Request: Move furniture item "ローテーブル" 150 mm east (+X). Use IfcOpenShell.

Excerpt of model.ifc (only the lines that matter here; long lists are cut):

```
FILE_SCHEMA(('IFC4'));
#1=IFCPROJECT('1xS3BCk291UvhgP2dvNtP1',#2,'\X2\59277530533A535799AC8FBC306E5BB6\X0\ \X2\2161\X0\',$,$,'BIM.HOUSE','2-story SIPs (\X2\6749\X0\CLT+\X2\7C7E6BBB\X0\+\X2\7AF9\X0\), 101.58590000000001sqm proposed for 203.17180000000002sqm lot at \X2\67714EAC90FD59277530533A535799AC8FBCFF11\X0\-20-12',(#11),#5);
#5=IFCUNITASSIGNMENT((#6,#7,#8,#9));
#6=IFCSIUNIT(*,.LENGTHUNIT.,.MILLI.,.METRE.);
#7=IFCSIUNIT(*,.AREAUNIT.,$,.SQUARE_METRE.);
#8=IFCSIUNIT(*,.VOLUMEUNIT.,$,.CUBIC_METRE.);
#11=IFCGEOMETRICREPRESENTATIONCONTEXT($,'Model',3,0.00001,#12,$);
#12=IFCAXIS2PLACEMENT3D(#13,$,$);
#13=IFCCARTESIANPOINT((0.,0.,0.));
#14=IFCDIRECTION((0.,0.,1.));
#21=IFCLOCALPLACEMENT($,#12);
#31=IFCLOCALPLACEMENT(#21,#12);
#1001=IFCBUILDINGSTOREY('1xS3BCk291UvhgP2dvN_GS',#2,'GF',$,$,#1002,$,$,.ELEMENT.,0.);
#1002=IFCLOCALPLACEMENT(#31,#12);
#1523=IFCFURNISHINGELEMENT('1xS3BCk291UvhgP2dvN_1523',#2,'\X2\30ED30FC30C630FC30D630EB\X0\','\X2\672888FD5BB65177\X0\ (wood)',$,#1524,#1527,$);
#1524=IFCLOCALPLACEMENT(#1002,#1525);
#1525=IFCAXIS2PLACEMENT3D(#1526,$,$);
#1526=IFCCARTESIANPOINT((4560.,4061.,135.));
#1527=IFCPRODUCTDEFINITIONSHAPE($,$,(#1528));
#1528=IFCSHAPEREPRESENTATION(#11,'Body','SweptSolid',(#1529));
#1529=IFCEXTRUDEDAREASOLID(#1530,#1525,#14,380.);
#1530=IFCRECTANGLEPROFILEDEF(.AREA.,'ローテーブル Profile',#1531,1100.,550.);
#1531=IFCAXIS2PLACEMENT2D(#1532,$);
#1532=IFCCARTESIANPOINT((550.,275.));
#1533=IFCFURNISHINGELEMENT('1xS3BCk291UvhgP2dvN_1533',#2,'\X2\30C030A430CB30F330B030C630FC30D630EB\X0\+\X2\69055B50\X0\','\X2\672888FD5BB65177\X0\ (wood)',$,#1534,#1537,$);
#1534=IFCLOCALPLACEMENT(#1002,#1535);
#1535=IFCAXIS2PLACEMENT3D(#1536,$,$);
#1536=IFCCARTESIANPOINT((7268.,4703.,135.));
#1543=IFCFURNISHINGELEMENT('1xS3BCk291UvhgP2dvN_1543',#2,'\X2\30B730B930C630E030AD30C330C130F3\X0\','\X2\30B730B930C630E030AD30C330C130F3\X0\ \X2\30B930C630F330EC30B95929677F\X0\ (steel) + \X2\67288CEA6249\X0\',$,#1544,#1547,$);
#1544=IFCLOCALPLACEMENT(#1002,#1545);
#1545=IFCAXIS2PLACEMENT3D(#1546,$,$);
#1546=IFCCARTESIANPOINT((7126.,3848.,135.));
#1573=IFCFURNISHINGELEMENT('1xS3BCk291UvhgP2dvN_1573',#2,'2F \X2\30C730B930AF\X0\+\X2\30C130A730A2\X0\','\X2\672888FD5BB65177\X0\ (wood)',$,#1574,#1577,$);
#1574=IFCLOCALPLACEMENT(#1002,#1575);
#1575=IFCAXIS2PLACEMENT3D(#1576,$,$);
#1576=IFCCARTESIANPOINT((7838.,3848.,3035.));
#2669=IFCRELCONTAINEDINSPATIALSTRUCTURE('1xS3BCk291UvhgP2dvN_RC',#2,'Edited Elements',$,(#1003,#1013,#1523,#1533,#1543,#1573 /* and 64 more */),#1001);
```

```python
import ifcopenshell
import ifcopenshell.api.geometry
import ifcopenshell.util.placement
import ifcopenshell.util.unit

model = ifcopenshell.open("model.ifc")
unit_scale = ifcopenshell.util.unit.calculate_unit_scale(model)

item = model.by_id(1523)
matrix = ifcopenshell.util.placement.get_local_placement(item.ObjectPlacement)
matrix[0, 3] += 0.15 / unit_scale
ifcopenshell.api.geometry.edit_object_placement(model, product=item, matrix=matrix, is_si=False)

print(ifcopenshell.util.placement.get_local_placement(item.ObjectPlacement).round(3) + 0.0)

model.write("model-out.ifc")
```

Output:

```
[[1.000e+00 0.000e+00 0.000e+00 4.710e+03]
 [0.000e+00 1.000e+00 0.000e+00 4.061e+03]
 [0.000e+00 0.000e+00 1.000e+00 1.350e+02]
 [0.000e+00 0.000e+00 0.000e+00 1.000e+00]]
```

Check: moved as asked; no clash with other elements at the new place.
